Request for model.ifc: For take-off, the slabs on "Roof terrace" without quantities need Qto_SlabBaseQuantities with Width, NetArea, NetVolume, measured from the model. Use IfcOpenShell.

First a look at what the model holds.

```python
import ifcopenshell
import ifcopenshell.util.element
import ifcopenshell.util.unit

model = ifcopenshell.open("model.ifc")
print(model.schema)
for unit_type in ("LENGTHUNIT", "AREAUNIT", "VOLUMEUNIT"):
    print(unit_type, ifcopenshell.util.unit.calculate_unit_scale(model, unit_type))
storey = next(s for s in model.by_type("IfcBuildingStorey") if s.Name == "Roof terrace")
slabs = [e for e in ifcopenshell.util.element.get_decomposition(storey) if e.is_a("IfcSlab")]
for e in sorted(slabs, key=lambda e: e.id()):
    print(e.id(), e.is_a(), e.Name, list(ifcopenshell.util.element.get_psets(e, qtos_only=True)), sep=" | ")
```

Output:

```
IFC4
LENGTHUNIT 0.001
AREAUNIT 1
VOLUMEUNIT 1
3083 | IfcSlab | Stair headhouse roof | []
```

```python
import ifcopenshell
import ifcopenshell.api.pset
import ifcopenshell.geom
import ifcopenshell.util.element
import ifcopenshell.util.shape
import ifcopenshell.util.unit

model = ifcopenshell.open("model.ifc")
unit_scale = ifcopenshell.util.unit.calculate_unit_scale(model)
area_scale = ifcopenshell.util.unit.calculate_unit_scale(model, "AREAUNIT")
volume_scale = ifcopenshell.util.unit.calculate_unit_scale(model, "VOLUMEUNIT")
settings = ifcopenshell.geom.settings()

storey = next(s for s in model.by_type("IfcBuildingStorey") if s.Name == "Roof terrace")
slabs = [e for e in ifcopenshell.util.element.get_decomposition(storey) if e.is_a("IfcSlab")]

for e in sorted(slabs, key=lambda e: e.id()):
    if ifcopenshell.util.element.get_psets(e, qtos_only=True, should_inherit=False):
        continue
    # Geometry comes back in metres, in the element's own axes.
    shape = ifcopenshell.geom.create_shape(settings, e)
    values = {
        "Width": ifcopenshell.util.shape.get_z(shape.geometry) / unit_scale,
        "NetArea": ifcopenshell.util.shape.get_footprint_area(shape.geometry) / area_scale,
        "NetVolume": ifcopenshell.util.shape.get_volume(shape.geometry) / volume_scale,
    }
    qto = ifcopenshell.api.pset.add_qto(model, product=e, name="Qto_SlabBaseQuantities")
    ifcopenshell.api.pset.edit_qto(model, qto=qto, properties=values)
    print(e.id(), {k: round(v, 3) for k, v in values.items()})

model.write("model-out.ifc")
```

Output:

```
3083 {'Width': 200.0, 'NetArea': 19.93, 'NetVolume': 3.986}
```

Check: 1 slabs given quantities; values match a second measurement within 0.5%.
